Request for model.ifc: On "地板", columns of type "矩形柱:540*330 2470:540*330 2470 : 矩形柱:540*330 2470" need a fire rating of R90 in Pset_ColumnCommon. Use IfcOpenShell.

First a look at what the model holds.

```python
import ifcopenshell
import ifcopenshell.util.element

model = ifcopenshell.open("model.ifc")
print(model.schema)
storey = next(s for s in model.by_type("IfcBuildingStorey") if s.Name == "地板")
columns = [e for e in ifcopenshell.util.element.get_decomposition(storey) if e.is_a("IfcColumn")]
seen = {}
for e in columns:
    element_type = ifcopenshell.util.element.get_type(e)
    key = (element_type.Name if element_type != e and element_type else None, ifcopenshell.util.element.get_pset(e, "Pset_ColumnCommon", "FireRating"))
    seen[key] = seen.get(key, 0) + 1
for (name, value), count in sorted(seen.items(), key=str):
    print(count, "x", name, "|", value)
```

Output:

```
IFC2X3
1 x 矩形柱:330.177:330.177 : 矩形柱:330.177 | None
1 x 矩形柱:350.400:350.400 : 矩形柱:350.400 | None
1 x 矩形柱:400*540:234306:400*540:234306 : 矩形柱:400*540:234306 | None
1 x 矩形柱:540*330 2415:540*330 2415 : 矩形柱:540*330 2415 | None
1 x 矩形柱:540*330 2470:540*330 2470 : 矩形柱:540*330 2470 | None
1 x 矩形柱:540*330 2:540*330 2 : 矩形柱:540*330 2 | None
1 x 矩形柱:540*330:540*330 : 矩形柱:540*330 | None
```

```python
import ifcopenshell
import ifcopenshell.api.pset
import ifcopenshell.util.element

model = ifcopenshell.open("model.ifc")

storey = next(s for s in model.by_type("IfcBuildingStorey") if s.Name == "地板")
columns = [e for e in ifcopenshell.util.element.get_decomposition(storey) if e.is_a("IfcColumn")]

count = 0
for e in columns:
    element_type = ifcopenshell.util.element.get_type(e)
    if element_type in (None, e) or element_type.Name != "矩形柱:540*330 2470:540*330 2470 : 矩形柱:540*330 2470":
        continue
    # add_pset returns the element's existing set when there is one.
    pset = ifcopenshell.api.pset.add_pset(model, product=e, name="Pset_ColumnCommon")
    ifcopenshell.api.pset.edit_pset(model, pset=pset, properties={"FireRating": "R90"})
    count += 1

print(count, "columns updated")

model.write("model-out.ifc")
```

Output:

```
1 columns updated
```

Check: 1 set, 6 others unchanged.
